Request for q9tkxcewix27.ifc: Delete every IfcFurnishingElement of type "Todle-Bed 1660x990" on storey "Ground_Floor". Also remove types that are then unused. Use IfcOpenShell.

First a look at what the model holds.

```python
import ifcopenshell
import ifcopenshell.util.element

model = ifcopenshell.open("q9tkxcewix27.ifc")
print(model.schema)
storey = next(s for s in model.by_type("IfcBuildingStorey") if s.Name == "Ground_Floor")
furniture = [e for e in ifcopenshell.util.element.get_decomposition(storey) if e.is_a("IfcFurnishingElement")]
seen = {}
for e in furniture:
    element_type = ifcopenshell.util.element.get_type(e)
    name = element_type.Name if element_type not in (None, e) else None
    seen[name] = seen.get(name, 0) + 1
for name, count in sorted(seen.items(), key=str):
    print(count, "x", name)
```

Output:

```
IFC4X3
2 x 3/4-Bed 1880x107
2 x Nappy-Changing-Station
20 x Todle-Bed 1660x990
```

```python
import ifcopenshell
import ifcopenshell.api.root
import ifcopenshell.util.element

model = ifcopenshell.open("q9tkxcewix27.ifc")

storey = next(s for s in model.by_type("IfcBuildingStorey") if s.Name == "Ground_Floor")
furniture = [e for e in ifcopenshell.util.element.get_decomposition(storey) if e.is_a("IfcFurnishingElement")]
targets = [e for e in furniture if (t := ifcopenshell.util.element.get_type(e)) not in (None, e) and t.Name == "Todle-Bed 1660x990"]
types = {ifcopenshell.util.element.get_type(e) for e in targets} - {None, *targets}

for e in targets:
    ifcopenshell.api.root.remove_product(model, product=e)
print(len(targets), "removed")

unused = [t for t in types if not ifcopenshell.util.element.get_types(t)]
for t in unused:
    ifcopenshell.api.root.remove_product(model, product=t)
print(len(unused), "unused types removed")

model.write("q9tkxcewix27_v2.ifc")
```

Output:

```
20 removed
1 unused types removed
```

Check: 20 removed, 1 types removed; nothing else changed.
